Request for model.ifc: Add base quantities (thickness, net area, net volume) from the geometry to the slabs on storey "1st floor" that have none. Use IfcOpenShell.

First a look at what the model holds.

```python
import ifcopenshell
import ifcopenshell.util.element
import ifcopenshell.util.unit

model = ifcopenshell.open("model.ifc")
print(model.schema)
for unit_type in ("LENGTHUNIT", "AREAUNIT", "VOLUMEUNIT"):
    print(unit_type, ifcopenshell.util.unit.calculate_unit_scale(model, unit_type))
storey = next(s for s in model.by_type("IfcBuildingStorey") if s.Name == "1st floor")
slabs = [e for e in ifcopenshell.util.element.get_decomposition(storey) if e.is_a("IfcSlab")]
for e in sorted(slabs, key=lambda e: e.id()):
    print(e.id(), e.is_a(), e.Name, list(ifcopenshell.util.element.get_psets(e, qtos_only=True)), sep=" | ")
```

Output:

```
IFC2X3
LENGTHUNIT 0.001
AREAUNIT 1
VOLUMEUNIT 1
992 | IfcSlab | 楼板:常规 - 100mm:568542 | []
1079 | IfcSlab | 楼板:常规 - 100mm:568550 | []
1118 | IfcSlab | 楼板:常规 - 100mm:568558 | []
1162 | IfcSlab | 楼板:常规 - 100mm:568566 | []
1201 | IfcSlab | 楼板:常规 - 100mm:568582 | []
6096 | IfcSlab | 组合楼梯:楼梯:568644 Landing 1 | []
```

```python
import ifcopenshell
import ifcopenshell.api.pset
import ifcopenshell.geom
import ifcopenshell.util.element
import ifcopenshell.util.shape
import ifcopenshell.util.unit

model = ifcopenshell.open("model.ifc")
unit_scale = ifcopenshell.util.unit.calculate_unit_scale(model)
area_scale = ifcopenshell.util.unit.calculate_unit_scale(model, "AREAUNIT")
volume_scale = ifcopenshell.util.unit.calculate_unit_scale(model, "VOLUMEUNIT")
settings = ifcopenshell.geom.settings()

storey = next(s for s in model.by_type("IfcBuildingStorey") if s.Name == "1st floor")
slabs = [e for e in ifcopenshell.util.element.get_decomposition(storey) if e.is_a("IfcSlab")]

for e in sorted(slabs, key=lambda e: e.id()):
    if ifcopenshell.util.element.get_psets(e, qtos_only=True, should_inherit=False):
        continue
    # Geometry comes back in metres, in the element's own axes.
    shape = ifcopenshell.geom.create_shape(settings, e)
    values = {
        "Width": ifcopenshell.util.shape.get_z(shape.geometry) / unit_scale,
        "NetArea": ifcopenshell.util.shape.get_footprint_area(shape.geometry) / area_scale,
        "NetVolume": ifcopenshell.util.shape.get_volume(shape.geometry) / volume_scale,
    }
    qto = ifcopenshell.api.pset.add_qto(model, product=e, name="BaseQuantities")
    ifcopenshell.api.pset.edit_qto(model, qto=qto, properties=values)
    print(e.id(), {k: round(v, 3) for k, v in values.items()})

model.write("model_v2.ifc")
```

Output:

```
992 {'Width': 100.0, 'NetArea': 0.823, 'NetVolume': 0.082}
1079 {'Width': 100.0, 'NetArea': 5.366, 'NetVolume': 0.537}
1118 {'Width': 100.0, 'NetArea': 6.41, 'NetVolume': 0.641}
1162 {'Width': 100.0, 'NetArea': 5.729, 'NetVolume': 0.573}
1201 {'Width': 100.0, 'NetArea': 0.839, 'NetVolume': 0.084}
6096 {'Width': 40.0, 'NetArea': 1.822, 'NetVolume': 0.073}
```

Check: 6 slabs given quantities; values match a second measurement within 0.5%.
